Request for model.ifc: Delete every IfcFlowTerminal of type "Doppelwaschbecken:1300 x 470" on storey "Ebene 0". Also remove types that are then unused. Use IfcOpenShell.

First a look at what the model holds.

```python
import ifcopenshell
import ifcopenshell.util.element

model = ifcopenshell.open("model.ifc")
print(model.schema)
storey = next(s for s in model.by_type("IfcBuildingStorey") if s.Name == "Ebene 0")
terminals = [e for e in ifcopenshell.util.element.get_decomposition(storey) if e.is_a("IfcFlowTerminal")]
seen = {}
for e in terminals:
    element_type = ifcopenshell.util.element.get_type(e)
    name = element_type.Name if element_type not in (None, e) else None
    seen[name] = seen.get(name, 0) + 1
for name, count in sorted(seen.items(), key=str):
    print(count, "x", name)
```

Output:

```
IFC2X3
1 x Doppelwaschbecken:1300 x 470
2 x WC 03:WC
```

```python
import ifcopenshell
import ifcopenshell.api.root
import ifcopenshell.util.element

model = ifcopenshell.open("model.ifc")

storey = next(s for s in model.by_type("IfcBuildingStorey") if s.Name == "Ebene 0")
terminals = [e for e in ifcopenshell.util.element.get_decomposition(storey) if e.is_a("IfcFlowTerminal")]
targets = [e for e in terminals if (t := ifcopenshell.util.element.get_type(e)) not in (None, e) and t.Name == "Doppelwaschbecken:1300 x 470"]
types = {ifcopenshell.util.element.get_type(e) for e in targets} - {None, *targets}

for e in targets:
    ifcopenshell.api.root.remove_product(model, product=e)
print(len(targets), "removed")

unused = [t for t in types if not ifcopenshell.util.element.get_types(t)]
for t in unused:
    ifcopenshell.api.root.remove_product(model, product=t)
print(len(unused), "unused types removed")

model.write("model_v2.ifc")
```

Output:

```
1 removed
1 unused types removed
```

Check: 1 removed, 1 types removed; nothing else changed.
